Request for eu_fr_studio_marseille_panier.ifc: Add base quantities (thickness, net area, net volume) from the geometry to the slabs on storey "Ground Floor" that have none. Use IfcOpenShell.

First a look at what the model holds.

```python
import ifcopenshell
import ifcopenshell.util.element
import ifcopenshell.util.unit

model = ifcopenshell.open("eu_fr_studio_marseille_panier.ifc")
print(model.schema)
for unit_type in ("LENGTHUNIT", "AREAUNIT", "VOLUMEUNIT"):
    print(unit_type, ifcopenshell.util.unit.calculate_unit_scale(model, unit_type))
storey = next(s for s in model.by_type("IfcBuildingStorey") if s.Name == "Ground Floor")
slabs = [e for e in ifcopenshell.util.element.get_decomposition(storey) if e.is_a("IfcSlab")]
for e in sorted(slabs, key=lambda e: e.id()):
    print(e.id(), e.is_a(), e.Name, list(ifcopenshell.util.element.get_psets(e, qtos_only=True)), sep=" | ")
```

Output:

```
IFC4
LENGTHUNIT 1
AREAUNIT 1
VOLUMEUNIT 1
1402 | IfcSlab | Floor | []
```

```python
import ifcopenshell
import ifcopenshell.api.pset
import ifcopenshell.geom
import ifcopenshell.util.element
import ifcopenshell.util.shape
import ifcopenshell.util.unit

model = ifcopenshell.open("eu_fr_studio_marseille_panier.ifc")
unit_scale = ifcopenshell.util.unit.calculate_unit_scale(model)
area_scale = ifcopenshell.util.unit.calculate_unit_scale(model, "AREAUNIT")
volume_scale = ifcopenshell.util.unit.calculate_unit_scale(model, "VOLUMEUNIT")
settings = ifcopenshell.geom.settings()

storey = next(s for s in model.by_type("IfcBuildingStorey") if s.Name == "Ground Floor")
slabs = [e for e in ifcopenshell.util.element.get_decomposition(storey) if e.is_a("IfcSlab")]

for e in sorted(slabs, key=lambda e: e.id()):
    if ifcopenshell.util.element.get_psets(e, qtos_only=True, should_inherit=False):
        continue
    # Geometry comes back in metres, in the element's own axes.
    shape = ifcopenshell.geom.create_shape(settings, e)
    values = {
        "Width": ifcopenshell.util.shape.get_z(shape.geometry) / unit_scale,
        "NetArea": ifcopenshell.util.shape.get_footprint_area(shape.geometry) / area_scale,
        "NetVolume": ifcopenshell.util.shape.get_volume(shape.geometry) / volume_scale,
    }
    qto = ifcopenshell.api.pset.add_qto(model, product=e, name="Qto_SlabBaseQuantities")
    ifcopenshell.api.pset.edit_qto(model, qto=qto, properties=values)
    print(e.id(), {k: round(v, 3) for k, v in values.items()})

model.write("eu_fr_studio_marseille_panier_rev.ifc")
```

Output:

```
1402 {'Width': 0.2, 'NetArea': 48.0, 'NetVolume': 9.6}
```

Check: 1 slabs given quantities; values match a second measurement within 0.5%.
